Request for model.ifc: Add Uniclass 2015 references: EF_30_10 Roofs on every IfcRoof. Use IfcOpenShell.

First a look at what the model holds.

```python
import ifcopenshell

model = ifcopenshell.open("model.ifc")
print(model.schema)
print("classifications:", [c.Name for c in model.by_type("IfcClassification")])
for ifc_class in ("IfcDoor", "IfcRoof", "IfcStair", "IfcWall", "IfcWindow"):
    print(ifc_class, len(model.by_type(ifc_class)))
```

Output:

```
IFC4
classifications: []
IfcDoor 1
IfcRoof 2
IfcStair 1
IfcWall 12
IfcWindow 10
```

```python
import ifcopenshell
import ifcopenshell.api.classification

model = ifcopenshell.open("model.ifc")

system = ifcopenshell.api.classification.add_classification(model, classification="Uniclass 2015")

codes = {
    "IfcRoof": ("EF_30_10", "Roofs"),
}
for ifc_class, (code, name) in codes.items():
    products = model.by_type(ifc_class)
    ifcopenshell.api.classification.add_reference(
        model, products=products, classification=system, identification=code, name=name
    )
    print(code, len(products))

model.write("model_rev.ifc")
```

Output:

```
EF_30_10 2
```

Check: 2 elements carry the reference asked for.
